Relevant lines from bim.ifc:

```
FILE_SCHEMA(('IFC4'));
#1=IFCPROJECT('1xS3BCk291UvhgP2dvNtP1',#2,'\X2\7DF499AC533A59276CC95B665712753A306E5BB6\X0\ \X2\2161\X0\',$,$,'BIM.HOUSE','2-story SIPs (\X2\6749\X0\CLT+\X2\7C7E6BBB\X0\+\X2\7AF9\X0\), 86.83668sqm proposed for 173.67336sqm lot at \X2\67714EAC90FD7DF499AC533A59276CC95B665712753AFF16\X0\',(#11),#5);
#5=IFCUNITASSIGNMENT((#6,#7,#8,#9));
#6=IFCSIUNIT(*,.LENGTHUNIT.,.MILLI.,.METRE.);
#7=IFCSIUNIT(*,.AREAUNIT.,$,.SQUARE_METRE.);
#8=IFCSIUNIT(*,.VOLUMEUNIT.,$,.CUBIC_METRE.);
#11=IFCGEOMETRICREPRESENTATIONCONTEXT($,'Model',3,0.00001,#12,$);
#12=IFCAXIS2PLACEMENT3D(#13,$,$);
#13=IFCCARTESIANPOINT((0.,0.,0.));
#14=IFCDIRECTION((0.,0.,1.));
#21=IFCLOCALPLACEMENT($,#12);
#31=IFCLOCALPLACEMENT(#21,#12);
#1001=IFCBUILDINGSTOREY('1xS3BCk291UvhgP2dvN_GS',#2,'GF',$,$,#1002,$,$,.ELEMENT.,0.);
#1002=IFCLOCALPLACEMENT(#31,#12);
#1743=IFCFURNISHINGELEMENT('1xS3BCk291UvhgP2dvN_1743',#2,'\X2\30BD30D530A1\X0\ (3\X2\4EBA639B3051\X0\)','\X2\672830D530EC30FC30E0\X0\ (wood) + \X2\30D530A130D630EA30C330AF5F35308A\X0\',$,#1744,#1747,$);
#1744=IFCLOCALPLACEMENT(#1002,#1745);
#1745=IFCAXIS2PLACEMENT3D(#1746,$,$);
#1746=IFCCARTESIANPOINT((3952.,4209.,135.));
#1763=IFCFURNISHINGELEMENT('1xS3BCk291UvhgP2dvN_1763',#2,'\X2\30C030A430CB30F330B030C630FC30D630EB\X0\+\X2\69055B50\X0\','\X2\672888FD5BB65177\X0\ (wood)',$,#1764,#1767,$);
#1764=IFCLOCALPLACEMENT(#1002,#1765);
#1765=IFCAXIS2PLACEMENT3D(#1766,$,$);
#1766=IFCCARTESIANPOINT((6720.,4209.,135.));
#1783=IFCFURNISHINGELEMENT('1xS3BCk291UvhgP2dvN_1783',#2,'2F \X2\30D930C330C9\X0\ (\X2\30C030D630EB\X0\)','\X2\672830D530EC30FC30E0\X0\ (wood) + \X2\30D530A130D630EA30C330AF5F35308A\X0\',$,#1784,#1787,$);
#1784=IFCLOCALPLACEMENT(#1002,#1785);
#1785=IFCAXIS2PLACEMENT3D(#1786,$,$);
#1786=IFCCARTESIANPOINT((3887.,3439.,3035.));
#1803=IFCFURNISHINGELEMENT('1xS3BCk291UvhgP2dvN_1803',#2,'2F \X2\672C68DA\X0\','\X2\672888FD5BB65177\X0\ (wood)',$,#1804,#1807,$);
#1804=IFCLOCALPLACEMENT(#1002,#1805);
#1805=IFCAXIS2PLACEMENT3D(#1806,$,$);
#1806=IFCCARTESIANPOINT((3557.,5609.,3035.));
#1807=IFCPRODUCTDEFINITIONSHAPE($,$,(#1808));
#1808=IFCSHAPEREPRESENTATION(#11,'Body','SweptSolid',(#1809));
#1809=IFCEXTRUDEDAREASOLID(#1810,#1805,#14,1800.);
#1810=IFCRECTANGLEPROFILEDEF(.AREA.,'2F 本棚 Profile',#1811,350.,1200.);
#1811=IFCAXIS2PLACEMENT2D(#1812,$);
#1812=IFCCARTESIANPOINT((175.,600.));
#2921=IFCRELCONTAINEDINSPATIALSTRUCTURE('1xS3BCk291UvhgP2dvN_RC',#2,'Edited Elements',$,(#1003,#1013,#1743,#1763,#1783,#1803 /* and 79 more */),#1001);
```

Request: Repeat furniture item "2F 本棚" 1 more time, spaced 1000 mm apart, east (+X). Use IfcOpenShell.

```python
import numpy as np
import ifcopenshell
import ifcopenshell.api.geometry
import ifcopenshell.api.root
import ifcopenshell.util.element
import ifcopenshell.util.placement
import ifcopenshell.util.unit

model = ifcopenshell.open("bim.ifc")
unit_scale = ifcopenshell.util.unit.calculate_unit_scale(model)


def reuse_history(source, copy):
    """copy_class also copies each property set's owner history, people and application; keep the originals."""
    for rel in copy.IsDefinedBy:
        if rel.is_a("IfcRelDefinesByProperties") and (history := rel.RelatingPropertyDefinition.OwnerHistory):
            rel.RelatingPropertyDefinition.OwnerHistory = source.OwnerHistory
            ifcopenshell.util.element.remove_deep2(model, history)


source = model.by_guid("1xS3BCk291UvhgP2dvN_1803")
base = ifcopenshell.util.placement.get_local_placement(source.ObjectPlacement)
step = np.array([1.0, 0.0, 0.0]) * 1 / unit_scale

for i in range(1, 2):
    copy = ifcopenshell.api.root.copy_class(model, product=source)
    copy.Representation = ifcopenshell.util.element.copy_deep(
        model, source.Representation, exclude=["IfcGeometricRepresentationContext", "IfcRepresentationMap"]
    )
    reuse_history(source, copy)
    matrix = base.copy()
    matrix[:3, 3] += i * step
    print("added at", matrix[:3, 3].round(3) + 0.0)
    ifcopenshell.api.geometry.edit_object_placement(model, product=copy, matrix=matrix, is_si=False)

model.write("bim_rev.ifc")
```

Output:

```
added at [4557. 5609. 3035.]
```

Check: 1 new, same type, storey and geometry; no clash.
